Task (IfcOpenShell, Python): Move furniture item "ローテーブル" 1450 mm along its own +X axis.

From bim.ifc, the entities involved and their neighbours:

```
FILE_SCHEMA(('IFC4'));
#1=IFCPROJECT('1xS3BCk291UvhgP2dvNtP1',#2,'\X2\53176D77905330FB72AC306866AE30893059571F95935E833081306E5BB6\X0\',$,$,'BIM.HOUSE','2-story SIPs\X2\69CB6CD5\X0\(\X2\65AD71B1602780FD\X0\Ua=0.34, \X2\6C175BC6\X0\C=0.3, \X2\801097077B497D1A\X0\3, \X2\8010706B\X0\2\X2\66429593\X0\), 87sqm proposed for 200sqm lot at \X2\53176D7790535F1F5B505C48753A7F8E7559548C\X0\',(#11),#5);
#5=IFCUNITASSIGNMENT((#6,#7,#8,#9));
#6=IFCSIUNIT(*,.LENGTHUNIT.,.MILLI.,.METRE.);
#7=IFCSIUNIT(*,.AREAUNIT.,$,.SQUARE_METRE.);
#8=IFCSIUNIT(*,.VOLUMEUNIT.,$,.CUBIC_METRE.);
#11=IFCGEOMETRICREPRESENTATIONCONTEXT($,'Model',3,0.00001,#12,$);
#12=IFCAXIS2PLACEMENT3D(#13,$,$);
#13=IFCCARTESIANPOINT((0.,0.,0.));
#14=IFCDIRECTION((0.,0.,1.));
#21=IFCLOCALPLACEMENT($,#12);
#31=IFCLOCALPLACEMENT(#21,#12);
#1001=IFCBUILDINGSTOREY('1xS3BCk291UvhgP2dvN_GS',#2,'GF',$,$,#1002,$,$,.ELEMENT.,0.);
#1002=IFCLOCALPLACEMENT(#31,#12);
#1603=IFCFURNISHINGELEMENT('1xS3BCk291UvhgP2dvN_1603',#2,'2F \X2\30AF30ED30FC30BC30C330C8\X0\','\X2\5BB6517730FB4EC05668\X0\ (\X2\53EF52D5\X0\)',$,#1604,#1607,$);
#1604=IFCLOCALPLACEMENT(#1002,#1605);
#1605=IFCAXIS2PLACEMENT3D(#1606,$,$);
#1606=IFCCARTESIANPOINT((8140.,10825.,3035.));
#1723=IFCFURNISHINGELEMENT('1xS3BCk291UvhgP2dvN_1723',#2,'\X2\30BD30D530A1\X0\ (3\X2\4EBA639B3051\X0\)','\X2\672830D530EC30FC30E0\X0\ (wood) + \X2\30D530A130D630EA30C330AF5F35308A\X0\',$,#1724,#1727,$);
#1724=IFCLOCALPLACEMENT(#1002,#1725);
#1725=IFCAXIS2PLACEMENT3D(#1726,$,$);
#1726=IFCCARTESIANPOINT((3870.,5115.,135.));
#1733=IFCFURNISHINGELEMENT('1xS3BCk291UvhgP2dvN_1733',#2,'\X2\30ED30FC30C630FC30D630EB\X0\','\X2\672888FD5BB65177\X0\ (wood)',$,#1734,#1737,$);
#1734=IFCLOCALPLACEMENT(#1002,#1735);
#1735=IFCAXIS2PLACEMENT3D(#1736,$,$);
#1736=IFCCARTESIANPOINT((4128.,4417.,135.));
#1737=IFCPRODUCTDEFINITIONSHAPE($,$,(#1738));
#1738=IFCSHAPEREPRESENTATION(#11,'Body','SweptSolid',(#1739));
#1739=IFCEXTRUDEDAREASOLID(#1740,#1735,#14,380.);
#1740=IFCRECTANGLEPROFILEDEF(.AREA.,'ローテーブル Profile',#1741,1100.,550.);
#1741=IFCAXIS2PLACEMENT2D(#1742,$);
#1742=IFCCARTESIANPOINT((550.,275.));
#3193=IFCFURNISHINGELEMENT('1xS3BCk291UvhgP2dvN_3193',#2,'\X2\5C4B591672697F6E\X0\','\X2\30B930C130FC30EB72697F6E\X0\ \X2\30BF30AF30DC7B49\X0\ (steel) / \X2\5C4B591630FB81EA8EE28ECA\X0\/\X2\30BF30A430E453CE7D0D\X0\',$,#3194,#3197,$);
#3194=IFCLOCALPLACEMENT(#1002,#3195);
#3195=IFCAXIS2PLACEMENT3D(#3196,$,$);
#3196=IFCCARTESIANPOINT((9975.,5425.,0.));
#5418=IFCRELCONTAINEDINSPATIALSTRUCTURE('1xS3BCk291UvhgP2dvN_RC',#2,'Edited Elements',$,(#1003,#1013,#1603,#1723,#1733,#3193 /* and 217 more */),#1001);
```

```python
import ifcopenshell
import ifcopenshell.api.geometry
import ifcopenshell.util.placement
import ifcopenshell.util.unit

model = ifcopenshell.open("bim.ifc")
unit_scale = ifcopenshell.util.unit.calculate_unit_scale(model)

item = model.by_guid("1xS3BCk291UvhgP2dvN_1733")
matrix = ifcopenshell.util.placement.get_local_placement(item.ObjectPlacement)
matrix[:3, 3] += matrix[:3, 0] * 1.45 / unit_scale
ifcopenshell.api.geometry.edit_object_placement(model, product=item, matrix=matrix, is_si=False)

print(ifcopenshell.util.placement.get_local_placement(item.ObjectPlacement).round(3) + 0.0)

model.write("bim_rev.ifc")
```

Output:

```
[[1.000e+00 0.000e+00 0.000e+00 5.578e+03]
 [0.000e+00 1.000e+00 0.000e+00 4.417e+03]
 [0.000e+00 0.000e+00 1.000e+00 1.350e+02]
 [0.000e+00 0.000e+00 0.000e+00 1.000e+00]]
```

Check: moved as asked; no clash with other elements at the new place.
